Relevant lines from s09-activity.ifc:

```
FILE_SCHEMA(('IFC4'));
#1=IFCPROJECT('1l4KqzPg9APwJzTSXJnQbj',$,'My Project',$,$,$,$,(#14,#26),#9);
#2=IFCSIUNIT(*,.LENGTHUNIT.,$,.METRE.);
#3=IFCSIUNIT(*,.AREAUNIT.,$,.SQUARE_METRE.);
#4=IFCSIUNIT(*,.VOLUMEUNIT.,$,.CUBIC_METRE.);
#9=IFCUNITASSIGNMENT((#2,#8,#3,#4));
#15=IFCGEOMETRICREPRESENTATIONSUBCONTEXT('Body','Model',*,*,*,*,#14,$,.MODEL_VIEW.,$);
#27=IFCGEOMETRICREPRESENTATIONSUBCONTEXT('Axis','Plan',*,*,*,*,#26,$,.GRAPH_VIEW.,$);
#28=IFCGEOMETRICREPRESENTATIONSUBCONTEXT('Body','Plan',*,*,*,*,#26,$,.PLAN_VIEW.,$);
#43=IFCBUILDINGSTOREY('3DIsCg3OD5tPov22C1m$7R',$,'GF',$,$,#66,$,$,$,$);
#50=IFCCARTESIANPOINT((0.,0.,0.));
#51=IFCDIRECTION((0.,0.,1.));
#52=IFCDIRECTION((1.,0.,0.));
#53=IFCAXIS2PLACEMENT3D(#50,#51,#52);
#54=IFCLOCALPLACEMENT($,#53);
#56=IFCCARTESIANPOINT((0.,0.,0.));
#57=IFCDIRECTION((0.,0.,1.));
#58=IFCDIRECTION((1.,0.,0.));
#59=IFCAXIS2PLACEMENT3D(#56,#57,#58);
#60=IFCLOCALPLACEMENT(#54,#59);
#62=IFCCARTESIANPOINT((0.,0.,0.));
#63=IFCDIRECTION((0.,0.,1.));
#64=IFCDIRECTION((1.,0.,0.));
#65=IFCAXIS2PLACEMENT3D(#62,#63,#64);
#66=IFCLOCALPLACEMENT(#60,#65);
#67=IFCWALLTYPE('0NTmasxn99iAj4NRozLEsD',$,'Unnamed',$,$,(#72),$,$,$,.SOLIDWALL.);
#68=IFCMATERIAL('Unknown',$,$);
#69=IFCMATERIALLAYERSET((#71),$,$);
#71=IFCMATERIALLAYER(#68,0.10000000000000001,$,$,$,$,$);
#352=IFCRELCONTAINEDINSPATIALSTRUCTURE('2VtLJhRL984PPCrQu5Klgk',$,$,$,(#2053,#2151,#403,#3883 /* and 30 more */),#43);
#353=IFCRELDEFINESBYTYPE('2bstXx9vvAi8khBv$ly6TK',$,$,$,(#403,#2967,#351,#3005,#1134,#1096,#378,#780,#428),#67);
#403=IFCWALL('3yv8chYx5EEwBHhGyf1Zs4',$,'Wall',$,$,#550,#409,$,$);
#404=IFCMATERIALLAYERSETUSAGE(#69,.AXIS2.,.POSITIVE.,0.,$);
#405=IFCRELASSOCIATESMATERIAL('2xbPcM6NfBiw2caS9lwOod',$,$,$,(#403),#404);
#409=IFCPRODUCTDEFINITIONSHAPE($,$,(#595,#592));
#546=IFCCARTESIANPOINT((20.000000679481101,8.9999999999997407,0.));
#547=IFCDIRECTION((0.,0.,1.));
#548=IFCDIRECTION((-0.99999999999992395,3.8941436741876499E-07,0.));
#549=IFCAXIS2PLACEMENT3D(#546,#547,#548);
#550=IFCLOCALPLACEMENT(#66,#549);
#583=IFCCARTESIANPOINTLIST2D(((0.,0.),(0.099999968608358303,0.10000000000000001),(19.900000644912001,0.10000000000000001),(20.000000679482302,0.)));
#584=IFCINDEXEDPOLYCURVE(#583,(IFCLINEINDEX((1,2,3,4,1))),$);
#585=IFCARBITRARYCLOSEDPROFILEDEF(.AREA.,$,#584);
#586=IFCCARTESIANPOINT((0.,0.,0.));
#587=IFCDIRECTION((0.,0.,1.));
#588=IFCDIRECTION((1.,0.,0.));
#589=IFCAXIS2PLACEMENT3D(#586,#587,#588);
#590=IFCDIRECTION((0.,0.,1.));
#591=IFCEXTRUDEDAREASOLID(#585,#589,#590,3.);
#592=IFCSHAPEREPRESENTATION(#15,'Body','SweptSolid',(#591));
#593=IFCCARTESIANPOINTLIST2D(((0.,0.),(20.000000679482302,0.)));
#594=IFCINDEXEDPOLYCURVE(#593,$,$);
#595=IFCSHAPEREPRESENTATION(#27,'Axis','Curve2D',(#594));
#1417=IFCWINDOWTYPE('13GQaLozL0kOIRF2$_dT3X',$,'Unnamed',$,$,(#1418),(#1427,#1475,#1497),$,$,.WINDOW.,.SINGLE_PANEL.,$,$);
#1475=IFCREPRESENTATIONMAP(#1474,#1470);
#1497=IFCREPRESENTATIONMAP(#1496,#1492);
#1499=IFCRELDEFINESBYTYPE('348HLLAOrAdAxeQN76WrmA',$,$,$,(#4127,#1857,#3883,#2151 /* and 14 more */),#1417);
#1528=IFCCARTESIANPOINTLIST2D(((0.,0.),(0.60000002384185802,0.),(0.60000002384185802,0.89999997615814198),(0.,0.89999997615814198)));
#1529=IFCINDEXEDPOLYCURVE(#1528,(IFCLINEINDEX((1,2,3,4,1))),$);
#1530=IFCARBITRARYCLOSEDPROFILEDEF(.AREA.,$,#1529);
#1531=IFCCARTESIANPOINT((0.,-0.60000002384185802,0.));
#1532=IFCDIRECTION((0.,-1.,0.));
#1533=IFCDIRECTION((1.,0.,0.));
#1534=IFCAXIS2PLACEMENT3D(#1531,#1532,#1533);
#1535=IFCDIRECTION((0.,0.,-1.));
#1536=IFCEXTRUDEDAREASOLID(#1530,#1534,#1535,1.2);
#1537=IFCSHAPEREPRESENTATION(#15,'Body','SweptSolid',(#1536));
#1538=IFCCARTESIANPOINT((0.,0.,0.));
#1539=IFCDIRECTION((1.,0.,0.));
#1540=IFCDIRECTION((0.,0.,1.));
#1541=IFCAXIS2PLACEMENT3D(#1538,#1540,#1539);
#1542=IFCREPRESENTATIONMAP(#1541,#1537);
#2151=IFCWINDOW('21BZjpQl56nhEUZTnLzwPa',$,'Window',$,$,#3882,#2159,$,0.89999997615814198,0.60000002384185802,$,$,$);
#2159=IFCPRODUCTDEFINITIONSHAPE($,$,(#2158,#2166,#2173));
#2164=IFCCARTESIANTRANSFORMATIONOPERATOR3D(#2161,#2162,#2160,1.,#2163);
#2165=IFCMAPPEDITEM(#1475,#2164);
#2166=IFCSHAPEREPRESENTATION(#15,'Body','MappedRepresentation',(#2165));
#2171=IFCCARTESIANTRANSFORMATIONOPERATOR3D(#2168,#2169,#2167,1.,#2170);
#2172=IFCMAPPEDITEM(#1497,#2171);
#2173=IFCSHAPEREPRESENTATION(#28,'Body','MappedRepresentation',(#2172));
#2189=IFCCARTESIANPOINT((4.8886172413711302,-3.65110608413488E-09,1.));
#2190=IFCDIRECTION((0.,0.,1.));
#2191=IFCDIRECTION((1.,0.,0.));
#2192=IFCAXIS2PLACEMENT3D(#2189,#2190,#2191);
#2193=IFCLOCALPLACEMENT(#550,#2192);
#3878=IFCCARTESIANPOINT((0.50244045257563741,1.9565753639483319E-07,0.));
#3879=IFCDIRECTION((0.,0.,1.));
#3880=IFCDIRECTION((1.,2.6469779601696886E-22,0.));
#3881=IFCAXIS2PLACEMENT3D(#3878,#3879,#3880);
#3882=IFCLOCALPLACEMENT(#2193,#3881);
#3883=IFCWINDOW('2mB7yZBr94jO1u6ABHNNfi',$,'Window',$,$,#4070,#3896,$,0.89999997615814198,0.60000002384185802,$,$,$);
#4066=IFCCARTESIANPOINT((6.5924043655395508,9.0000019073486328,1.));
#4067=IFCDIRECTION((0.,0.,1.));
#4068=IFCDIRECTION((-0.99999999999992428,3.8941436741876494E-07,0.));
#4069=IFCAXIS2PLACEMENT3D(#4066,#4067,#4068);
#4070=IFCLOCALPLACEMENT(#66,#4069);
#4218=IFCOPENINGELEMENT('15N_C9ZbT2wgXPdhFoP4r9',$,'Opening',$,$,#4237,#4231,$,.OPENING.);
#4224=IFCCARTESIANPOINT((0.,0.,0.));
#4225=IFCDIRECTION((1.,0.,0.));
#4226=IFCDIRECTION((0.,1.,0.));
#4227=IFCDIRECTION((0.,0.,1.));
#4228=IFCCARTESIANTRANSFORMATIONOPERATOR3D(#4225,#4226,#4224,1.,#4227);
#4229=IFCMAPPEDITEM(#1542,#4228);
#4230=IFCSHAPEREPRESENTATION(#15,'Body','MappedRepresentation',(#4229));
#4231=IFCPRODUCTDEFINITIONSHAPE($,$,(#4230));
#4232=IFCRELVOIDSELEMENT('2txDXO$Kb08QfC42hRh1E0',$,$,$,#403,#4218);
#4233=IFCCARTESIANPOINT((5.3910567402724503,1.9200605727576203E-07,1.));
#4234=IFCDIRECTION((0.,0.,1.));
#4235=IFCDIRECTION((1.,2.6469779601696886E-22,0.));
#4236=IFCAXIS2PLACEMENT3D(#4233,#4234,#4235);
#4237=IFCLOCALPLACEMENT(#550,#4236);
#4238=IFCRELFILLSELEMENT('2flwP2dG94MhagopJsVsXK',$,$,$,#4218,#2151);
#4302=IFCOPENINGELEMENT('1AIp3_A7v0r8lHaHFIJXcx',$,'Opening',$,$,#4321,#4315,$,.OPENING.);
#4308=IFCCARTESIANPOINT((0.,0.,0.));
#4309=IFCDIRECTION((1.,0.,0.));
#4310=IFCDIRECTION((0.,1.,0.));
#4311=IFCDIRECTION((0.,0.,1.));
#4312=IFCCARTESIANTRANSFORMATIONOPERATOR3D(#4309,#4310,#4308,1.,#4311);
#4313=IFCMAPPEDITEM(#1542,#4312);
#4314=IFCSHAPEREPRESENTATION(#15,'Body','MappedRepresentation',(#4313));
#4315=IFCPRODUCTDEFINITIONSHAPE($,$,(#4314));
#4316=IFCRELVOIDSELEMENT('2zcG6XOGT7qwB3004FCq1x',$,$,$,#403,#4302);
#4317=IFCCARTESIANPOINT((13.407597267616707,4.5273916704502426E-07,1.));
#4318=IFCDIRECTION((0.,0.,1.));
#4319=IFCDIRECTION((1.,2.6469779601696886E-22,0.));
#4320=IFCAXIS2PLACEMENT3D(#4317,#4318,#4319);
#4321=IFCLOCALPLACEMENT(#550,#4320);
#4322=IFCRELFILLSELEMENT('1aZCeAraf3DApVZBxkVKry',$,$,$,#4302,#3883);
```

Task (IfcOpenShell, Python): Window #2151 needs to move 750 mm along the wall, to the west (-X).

```python
import ifcopenshell
import ifcopenshell.api.geometry
import ifcopenshell.util.placement

model = ifcopenshell.open("s09-activity.ifc")

window = model.by_id(2151)
opening = window.FillsVoids[0].RelatingOpeningElement
wall = opening.VoidsElements[0].RelatingBuildingElement

wall_matrix = ifcopenshell.util.placement.get_local_placement(wall.ObjectPlacement)
shift = wall_matrix[:3, 0] * 0.75
before = ifcopenshell.util.placement.get_local_placement(window.ObjectPlacement)[:3, 3].copy()

# The window is not placed relative to its opening, so move both.
for product in (opening, window):
    matrix = ifcopenshell.util.placement.get_local_placement(product.ObjectPlacement)
    matrix[:3, 3] += shift
    ifcopenshell.api.geometry.edit_object_placement(model, product=product, matrix=matrix, is_si=False)

after = ifcopenshell.util.placement.get_local_placement(window.ObjectPlacement)[:3, 3]
print("window moved by", (after - before).round(3) + 0.0)

model.write("s09-activity_v2.ifc")
```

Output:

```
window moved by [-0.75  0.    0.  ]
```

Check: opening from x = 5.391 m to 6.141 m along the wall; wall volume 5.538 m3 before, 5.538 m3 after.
